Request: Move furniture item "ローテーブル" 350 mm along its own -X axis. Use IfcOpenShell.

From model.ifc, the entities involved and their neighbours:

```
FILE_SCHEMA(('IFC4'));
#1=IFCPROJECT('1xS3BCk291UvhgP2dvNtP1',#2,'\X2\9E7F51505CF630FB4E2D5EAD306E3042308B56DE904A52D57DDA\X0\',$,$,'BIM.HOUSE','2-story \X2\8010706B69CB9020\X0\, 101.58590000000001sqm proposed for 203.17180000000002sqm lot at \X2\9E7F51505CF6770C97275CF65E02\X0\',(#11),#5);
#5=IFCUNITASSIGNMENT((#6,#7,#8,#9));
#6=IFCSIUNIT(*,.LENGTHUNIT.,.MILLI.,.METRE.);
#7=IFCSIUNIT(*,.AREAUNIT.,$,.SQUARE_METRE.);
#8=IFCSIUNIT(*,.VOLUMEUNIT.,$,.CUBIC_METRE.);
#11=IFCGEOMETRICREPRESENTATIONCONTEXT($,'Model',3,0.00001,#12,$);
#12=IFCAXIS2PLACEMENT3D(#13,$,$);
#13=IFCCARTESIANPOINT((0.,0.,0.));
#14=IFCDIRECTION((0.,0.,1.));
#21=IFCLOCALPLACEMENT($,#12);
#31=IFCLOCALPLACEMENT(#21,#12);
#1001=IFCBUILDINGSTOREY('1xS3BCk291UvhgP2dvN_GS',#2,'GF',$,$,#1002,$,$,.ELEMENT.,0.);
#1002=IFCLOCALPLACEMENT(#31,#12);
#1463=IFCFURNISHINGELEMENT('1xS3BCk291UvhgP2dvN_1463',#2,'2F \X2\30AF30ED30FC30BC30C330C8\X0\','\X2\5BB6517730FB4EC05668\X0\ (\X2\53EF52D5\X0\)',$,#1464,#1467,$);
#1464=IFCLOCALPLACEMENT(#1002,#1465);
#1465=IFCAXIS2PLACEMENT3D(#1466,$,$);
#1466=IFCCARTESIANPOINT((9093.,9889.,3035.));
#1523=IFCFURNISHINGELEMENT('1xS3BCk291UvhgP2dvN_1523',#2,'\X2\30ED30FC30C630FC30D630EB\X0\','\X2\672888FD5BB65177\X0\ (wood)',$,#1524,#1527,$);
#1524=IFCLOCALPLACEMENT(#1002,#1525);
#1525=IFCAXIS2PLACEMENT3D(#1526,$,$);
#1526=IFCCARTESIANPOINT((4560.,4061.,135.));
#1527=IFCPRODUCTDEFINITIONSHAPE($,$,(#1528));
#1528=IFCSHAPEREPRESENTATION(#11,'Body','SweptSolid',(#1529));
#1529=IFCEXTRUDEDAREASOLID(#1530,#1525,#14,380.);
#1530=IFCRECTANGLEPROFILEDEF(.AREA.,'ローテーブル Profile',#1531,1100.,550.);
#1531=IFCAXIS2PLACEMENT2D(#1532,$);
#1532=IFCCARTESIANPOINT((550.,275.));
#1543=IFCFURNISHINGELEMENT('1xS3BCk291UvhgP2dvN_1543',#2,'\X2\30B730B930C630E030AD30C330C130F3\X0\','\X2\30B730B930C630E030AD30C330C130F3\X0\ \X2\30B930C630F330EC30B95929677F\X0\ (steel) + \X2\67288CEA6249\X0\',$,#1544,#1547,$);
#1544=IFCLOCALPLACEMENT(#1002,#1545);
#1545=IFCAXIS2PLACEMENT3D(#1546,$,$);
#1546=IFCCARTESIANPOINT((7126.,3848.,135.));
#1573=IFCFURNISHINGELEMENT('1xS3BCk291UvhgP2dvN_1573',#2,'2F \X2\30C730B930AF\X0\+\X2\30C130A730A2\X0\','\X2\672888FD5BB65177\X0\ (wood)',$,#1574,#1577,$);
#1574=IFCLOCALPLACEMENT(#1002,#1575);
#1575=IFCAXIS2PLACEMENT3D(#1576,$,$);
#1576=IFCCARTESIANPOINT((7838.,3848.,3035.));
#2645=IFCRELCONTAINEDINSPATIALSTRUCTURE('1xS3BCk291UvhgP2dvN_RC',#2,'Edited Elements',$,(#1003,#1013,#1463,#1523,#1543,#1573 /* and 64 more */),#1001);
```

```python
import ifcopenshell
import ifcopenshell.api.geometry
import ifcopenshell.util.placement
import ifcopenshell.util.unit

model = ifcopenshell.open("model.ifc")
unit_scale = ifcopenshell.util.unit.calculate_unit_scale(model)

item = model.by_guid("1xS3BCk291UvhgP2dvN_1523")
matrix = ifcopenshell.util.placement.get_local_placement(item.ObjectPlacement)
matrix[:3, 3] -= matrix[:3, 0] * 0.35 / unit_scale
ifcopenshell.api.geometry.edit_object_placement(model, product=item, matrix=matrix, is_si=False)

print(ifcopenshell.util.placement.get_local_placement(item.ObjectPlacement).round(3) + 0.0)

model.write("model_v2.ifc")
```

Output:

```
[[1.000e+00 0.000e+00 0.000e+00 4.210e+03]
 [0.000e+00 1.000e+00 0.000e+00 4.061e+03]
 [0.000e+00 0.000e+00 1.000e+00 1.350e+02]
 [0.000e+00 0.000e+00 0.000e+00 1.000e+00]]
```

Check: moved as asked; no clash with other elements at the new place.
